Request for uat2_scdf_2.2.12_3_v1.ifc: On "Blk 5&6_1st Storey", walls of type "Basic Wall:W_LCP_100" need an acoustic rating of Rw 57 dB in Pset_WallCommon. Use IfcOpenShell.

First a look at what the model holds.

```python
import ifcopenshell
import ifcopenshell.util.element

model = ifcopenshell.open("uat2_scdf_2.2.12_3_v1.ifc")
print(model.schema)
storey = next(s for s in model.by_type("IfcBuildingStorey") if s.Name == "Blk 5&6_1st Storey")
walls = [e for e in ifcopenshell.util.element.get_decomposition(storey) if e.is_a("IfcWall")]
seen = {}
for e in walls:
    element_type = ifcopenshell.util.element.get_type(e)
    key = (element_type.Name if element_type != e and element_type else None, ifcopenshell.util.element.get_pset(e, "Pset_WallCommon", "AcousticRating"))
    seen[key] = seen.get(key, 0) + 1
for (name, value), count in sorted(seen.items(), key=str):
    print(count, "x", name, "|", value)
```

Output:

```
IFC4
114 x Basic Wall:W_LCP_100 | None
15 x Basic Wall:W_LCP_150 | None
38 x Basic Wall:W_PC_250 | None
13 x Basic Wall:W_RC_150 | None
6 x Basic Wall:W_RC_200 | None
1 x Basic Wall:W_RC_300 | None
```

```python
import ifcopenshell
import ifcopenshell.api.pset
import ifcopenshell.util.element

model = ifcopenshell.open("uat2_scdf_2.2.12_3_v1.ifc")

storey = next(s for s in model.by_type("IfcBuildingStorey") if s.Name == "Blk 5&6_1st Storey")
walls = [e for e in ifcopenshell.util.element.get_decomposition(storey) if e.is_a("IfcWall")]

count = 0
for e in walls:
    element_type = ifcopenshell.util.element.get_type(e)
    if element_type in (None, e) or element_type.Name != "Basic Wall:W_LCP_100":
        continue
    # add_pset returns the element's existing set when there is one.
    pset = ifcopenshell.api.pset.add_pset(model, product=e, name="Pset_WallCommon")
    ifcopenshell.api.pset.edit_pset(model, pset=pset, properties={"AcousticRating": "Rw 57 dB"})
    count += 1

print(count, "walls updated")

model.write("uat2_scdf_2.2.12_3_v1_rev.ifc")
```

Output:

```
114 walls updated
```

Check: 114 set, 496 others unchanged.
